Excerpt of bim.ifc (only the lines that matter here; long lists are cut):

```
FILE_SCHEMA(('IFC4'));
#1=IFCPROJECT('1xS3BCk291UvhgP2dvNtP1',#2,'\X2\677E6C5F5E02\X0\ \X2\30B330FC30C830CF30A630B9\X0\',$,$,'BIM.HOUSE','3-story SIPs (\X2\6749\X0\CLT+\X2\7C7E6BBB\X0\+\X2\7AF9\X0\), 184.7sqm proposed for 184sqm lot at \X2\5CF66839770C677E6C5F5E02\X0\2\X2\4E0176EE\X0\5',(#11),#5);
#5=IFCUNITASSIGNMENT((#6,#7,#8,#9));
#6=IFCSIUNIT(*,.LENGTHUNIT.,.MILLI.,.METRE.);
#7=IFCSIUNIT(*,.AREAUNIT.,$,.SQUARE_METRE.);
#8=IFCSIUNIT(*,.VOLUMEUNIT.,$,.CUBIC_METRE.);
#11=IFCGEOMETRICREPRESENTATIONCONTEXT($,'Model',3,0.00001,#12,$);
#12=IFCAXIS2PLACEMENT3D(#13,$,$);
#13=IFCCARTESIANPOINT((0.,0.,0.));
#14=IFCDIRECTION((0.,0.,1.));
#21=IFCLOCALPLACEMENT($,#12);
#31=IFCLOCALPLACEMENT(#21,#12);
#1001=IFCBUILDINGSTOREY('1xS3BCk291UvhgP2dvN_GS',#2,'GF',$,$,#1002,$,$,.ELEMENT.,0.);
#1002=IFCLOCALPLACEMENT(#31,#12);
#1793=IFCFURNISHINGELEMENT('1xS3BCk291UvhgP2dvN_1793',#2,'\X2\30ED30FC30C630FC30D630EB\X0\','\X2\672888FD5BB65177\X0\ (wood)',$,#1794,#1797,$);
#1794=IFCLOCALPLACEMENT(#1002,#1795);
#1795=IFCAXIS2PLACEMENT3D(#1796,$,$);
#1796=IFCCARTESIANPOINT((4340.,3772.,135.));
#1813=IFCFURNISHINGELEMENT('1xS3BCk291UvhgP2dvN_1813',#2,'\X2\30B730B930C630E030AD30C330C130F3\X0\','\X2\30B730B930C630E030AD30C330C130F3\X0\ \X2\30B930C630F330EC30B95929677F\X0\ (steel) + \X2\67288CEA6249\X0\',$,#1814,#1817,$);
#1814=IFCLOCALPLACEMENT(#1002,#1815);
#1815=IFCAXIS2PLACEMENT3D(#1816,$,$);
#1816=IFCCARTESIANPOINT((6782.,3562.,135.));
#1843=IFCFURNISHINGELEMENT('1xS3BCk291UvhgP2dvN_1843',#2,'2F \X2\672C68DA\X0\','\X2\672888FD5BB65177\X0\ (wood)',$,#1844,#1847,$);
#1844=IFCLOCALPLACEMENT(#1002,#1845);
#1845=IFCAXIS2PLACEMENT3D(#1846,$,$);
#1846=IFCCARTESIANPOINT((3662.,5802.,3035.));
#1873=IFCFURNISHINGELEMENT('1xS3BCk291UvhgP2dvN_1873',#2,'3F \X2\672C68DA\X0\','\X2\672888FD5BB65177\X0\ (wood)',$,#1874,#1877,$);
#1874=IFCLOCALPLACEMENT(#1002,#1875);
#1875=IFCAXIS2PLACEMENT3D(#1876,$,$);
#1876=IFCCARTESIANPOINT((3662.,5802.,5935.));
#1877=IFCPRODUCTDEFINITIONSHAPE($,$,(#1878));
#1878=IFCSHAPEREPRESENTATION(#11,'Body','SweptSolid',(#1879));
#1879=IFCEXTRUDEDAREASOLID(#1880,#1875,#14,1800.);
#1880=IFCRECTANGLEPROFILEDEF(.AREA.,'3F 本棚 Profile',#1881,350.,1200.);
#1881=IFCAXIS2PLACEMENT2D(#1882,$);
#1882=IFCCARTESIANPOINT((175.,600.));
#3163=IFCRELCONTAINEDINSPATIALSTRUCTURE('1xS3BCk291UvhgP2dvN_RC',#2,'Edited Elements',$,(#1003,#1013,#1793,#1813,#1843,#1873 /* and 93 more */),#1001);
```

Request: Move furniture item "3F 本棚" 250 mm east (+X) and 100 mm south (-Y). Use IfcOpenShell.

```python
import ifcopenshell
import ifcopenshell.api.geometry
import ifcopenshell.util.placement
import ifcopenshell.util.unit

model = ifcopenshell.open("bim.ifc")
unit_scale = ifcopenshell.util.unit.calculate_unit_scale(model)

item = model.by_guid("1xS3BCk291UvhgP2dvN_1873")
matrix = ifcopenshell.util.placement.get_local_placement(item.ObjectPlacement)
matrix[0, 3] += 0.25 / unit_scale
matrix[1, 3] -= 0.1 / unit_scale
ifcopenshell.api.geometry.edit_object_placement(model, product=item, matrix=matrix, is_si=False)

print(ifcopenshell.util.placement.get_local_placement(item.ObjectPlacement).round(3) + 0.0)

model.write("bim_updated.ifc")
```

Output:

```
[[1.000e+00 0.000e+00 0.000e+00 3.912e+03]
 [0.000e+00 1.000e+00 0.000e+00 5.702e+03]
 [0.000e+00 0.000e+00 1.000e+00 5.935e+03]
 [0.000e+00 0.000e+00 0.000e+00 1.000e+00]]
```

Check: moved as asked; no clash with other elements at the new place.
